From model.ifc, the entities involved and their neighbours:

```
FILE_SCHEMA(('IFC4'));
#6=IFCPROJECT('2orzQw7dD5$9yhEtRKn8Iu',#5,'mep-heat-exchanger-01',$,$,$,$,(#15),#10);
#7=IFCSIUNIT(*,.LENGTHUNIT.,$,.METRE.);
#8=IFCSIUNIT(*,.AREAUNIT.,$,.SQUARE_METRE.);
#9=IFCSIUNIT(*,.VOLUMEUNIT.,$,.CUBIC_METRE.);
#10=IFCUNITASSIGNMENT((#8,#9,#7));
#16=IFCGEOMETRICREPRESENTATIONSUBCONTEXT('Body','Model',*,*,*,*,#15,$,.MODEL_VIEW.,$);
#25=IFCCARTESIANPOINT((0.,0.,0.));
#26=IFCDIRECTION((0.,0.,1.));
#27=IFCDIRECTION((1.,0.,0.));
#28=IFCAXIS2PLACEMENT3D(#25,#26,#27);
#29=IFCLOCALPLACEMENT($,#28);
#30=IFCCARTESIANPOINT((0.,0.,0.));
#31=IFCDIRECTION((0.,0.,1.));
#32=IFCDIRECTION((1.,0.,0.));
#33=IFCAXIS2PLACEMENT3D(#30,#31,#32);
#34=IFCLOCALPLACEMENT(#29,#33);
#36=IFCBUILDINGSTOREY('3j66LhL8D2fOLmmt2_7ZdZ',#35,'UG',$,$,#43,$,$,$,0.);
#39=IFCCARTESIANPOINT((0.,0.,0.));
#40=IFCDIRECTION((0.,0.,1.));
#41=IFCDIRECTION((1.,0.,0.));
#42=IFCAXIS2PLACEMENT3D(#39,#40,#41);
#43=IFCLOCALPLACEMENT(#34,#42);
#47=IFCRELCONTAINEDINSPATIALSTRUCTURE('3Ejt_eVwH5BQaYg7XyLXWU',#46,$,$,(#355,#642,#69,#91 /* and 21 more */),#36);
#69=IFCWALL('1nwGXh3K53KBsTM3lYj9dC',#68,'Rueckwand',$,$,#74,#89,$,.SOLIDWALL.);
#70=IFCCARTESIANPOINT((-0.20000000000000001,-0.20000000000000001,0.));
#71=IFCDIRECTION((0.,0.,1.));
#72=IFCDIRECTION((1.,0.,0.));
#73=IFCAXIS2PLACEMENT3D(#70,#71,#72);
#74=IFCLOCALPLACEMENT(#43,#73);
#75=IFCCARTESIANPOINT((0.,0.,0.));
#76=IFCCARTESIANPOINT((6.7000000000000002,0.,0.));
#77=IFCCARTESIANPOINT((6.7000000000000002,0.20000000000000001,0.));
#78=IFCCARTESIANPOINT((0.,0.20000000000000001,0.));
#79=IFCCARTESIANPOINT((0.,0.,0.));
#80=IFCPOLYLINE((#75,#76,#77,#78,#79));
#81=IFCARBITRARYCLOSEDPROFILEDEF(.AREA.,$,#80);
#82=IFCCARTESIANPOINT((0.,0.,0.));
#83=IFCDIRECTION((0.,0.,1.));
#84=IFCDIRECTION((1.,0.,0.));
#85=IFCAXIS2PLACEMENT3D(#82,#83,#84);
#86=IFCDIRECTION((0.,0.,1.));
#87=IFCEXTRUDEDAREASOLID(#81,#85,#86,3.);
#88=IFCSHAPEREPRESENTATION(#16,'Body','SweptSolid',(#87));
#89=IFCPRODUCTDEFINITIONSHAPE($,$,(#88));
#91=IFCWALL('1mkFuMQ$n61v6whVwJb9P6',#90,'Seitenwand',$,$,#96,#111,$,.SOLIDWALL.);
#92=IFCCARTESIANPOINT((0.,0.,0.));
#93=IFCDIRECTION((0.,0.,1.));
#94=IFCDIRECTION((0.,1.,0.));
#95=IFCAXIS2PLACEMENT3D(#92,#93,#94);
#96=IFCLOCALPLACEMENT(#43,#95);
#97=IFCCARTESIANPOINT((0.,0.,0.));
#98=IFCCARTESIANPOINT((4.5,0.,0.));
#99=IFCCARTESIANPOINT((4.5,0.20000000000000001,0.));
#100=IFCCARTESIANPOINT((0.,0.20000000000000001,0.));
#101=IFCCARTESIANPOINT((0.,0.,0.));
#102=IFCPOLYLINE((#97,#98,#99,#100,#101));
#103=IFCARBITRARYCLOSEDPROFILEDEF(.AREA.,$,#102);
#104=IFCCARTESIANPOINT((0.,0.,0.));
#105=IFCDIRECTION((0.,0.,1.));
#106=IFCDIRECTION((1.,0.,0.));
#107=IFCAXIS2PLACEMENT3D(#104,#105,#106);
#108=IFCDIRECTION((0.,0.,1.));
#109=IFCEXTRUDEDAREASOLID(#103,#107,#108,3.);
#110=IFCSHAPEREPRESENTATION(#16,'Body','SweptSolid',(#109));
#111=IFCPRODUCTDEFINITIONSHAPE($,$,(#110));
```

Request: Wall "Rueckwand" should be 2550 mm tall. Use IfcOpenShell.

```python
import ifcopenshell
import ifcopenshell.geom
import ifcopenshell.util.representation
import ifcopenshell.util.shape
import ifcopenshell.util.unit

model = ifcopenshell.open("model.ifc")
unit_scale = ifcopenshell.util.unit.calculate_unit_scale(model)
settings = ifcopenshell.geom.settings()


def volume(element):
    """Net volume in cubic metres, openings subtracted."""
    shape = ifcopenshell.geom.create_shape(settings, element)
    return ifcopenshell.util.shape.get_volume(shape.geometry)


wall = model.by_guid("1nwGXh3K53KBsTM3lYj9dC")
before = volume(wall)

body = ifcopenshell.util.representation.get_representation(wall, "Model", "Body")
solid = body.Items[0]
old_height = solid.Depth
solid.Depth = 2.55 / unit_scale
after = volume(wall)

print(f"height {old_height:g} -> {solid.Depth:g}, volume {before:.3f} -> {after:.3f} m3")

model.write("model_edited.ifc")
```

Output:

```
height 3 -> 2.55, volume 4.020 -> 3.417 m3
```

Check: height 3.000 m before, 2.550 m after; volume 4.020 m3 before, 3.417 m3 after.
